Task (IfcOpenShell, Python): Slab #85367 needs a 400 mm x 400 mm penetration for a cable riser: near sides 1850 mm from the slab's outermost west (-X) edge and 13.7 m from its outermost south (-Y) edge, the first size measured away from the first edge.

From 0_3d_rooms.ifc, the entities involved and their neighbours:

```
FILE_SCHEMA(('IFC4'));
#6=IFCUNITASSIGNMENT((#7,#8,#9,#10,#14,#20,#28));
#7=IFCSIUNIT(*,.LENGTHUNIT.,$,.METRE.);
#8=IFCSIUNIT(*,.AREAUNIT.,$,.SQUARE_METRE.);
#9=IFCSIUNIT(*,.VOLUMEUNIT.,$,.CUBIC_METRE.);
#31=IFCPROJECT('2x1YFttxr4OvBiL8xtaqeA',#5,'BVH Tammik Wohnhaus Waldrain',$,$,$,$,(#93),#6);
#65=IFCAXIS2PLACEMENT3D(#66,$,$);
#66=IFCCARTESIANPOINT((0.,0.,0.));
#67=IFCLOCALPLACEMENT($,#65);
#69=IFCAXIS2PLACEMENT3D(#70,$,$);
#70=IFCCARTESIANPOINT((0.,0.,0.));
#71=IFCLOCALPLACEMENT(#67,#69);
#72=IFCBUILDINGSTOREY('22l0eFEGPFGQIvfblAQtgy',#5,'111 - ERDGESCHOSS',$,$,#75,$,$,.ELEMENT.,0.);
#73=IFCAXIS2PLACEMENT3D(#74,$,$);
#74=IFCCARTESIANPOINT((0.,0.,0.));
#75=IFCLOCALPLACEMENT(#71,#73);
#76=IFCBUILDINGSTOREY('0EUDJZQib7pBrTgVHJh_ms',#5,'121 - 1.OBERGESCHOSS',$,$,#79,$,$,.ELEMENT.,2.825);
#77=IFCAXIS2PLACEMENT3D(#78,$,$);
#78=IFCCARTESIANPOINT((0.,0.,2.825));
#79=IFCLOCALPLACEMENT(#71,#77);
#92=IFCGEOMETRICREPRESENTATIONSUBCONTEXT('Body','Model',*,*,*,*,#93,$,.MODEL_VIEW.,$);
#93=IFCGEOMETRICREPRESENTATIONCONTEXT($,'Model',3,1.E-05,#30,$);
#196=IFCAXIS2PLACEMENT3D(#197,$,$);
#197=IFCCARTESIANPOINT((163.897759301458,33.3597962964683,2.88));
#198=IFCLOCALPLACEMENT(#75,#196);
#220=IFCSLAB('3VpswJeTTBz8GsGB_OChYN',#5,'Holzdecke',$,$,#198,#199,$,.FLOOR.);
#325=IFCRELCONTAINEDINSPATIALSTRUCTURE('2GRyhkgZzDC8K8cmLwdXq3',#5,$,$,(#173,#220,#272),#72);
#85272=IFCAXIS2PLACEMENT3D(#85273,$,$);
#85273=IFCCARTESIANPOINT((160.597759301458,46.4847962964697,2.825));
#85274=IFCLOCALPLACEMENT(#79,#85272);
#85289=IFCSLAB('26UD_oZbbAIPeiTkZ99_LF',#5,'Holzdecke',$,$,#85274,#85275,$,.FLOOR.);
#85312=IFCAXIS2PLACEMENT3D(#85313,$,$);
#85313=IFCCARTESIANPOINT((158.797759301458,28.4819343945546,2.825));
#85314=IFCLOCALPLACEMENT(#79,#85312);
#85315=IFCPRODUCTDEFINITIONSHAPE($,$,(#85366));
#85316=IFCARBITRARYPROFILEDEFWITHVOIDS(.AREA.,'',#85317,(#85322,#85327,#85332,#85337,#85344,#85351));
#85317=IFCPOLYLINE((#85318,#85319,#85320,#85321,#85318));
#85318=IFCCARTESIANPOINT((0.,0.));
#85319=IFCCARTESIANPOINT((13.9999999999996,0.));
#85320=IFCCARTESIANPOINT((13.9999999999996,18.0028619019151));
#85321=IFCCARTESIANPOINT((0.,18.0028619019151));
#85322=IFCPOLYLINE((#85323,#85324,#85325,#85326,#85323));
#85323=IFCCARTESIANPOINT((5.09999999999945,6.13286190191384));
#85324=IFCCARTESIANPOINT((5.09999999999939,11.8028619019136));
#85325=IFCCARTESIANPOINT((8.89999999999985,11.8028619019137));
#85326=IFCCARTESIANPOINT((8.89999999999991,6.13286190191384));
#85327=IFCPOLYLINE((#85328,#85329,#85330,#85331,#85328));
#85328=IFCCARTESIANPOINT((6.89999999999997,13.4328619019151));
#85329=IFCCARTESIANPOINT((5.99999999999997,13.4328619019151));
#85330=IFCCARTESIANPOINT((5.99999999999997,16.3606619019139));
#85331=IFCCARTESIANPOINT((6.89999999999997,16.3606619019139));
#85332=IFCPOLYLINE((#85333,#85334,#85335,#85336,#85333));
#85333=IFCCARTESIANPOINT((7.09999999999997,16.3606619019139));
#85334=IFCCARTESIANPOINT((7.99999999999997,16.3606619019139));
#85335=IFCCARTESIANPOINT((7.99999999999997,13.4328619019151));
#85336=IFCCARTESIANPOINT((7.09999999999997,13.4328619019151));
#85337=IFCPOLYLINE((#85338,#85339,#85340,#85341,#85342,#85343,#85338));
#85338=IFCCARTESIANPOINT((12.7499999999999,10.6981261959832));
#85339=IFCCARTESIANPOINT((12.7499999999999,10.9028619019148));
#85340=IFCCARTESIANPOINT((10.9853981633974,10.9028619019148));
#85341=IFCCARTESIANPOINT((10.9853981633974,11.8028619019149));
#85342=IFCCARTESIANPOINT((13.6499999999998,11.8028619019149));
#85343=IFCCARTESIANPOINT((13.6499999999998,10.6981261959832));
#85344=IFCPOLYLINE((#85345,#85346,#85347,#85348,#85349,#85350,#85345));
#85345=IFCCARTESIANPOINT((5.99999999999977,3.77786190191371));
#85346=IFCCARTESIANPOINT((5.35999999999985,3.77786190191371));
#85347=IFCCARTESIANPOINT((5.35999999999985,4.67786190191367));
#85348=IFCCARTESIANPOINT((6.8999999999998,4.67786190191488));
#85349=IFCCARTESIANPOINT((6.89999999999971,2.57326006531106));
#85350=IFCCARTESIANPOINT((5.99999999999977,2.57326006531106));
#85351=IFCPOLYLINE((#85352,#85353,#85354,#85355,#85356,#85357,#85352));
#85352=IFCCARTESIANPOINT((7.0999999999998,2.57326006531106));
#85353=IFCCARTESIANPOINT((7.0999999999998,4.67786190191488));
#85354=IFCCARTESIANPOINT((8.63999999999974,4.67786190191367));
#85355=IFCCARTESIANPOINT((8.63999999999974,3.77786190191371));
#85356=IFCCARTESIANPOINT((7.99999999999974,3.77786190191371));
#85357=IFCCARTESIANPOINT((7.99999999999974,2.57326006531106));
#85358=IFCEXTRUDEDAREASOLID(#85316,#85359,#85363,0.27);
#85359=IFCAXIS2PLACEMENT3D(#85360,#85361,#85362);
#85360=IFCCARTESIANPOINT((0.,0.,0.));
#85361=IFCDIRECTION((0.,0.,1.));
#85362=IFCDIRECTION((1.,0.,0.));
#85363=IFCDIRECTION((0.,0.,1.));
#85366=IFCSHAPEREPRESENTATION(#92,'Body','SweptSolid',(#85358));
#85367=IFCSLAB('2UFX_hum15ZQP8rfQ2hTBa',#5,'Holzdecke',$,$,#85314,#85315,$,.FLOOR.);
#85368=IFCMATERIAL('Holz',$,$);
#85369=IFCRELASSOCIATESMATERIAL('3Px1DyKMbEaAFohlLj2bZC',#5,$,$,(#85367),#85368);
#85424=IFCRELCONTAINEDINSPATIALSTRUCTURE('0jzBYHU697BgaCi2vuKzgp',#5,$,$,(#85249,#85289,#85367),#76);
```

```python
import numpy as np
import ifcopenshell
import ifcopenshell.api.feature
import ifcopenshell.api.geometry
import ifcopenshell.api.root
import ifcopenshell.geom
import ifcopenshell.util.placement
import ifcopenshell.util.representation
import ifcopenshell.util.shape
import ifcopenshell.util.unit

model = ifcopenshell.open("0_3d_rooms.ifc")
unit_scale = ifcopenshell.util.unit.calculate_unit_scale(model)
settings = ifcopenshell.geom.settings()


def volume(element):
    """Net volume in cubic metres, openings subtracted."""
    shape = ifcopenshell.geom.create_shape(settings, element)
    return ifcopenshell.util.shape.get_volume(shape.geometry)


slab = model.by_id(85367)
before = volume(slab)

# Extent in the slab's own axes, in metres. The edges named are its -X and -Y sides.
slab_shape = ifcopenshell.geom.create_shape(settings, slab)
vertices = ifcopenshell.util.shape.get_vertices(slab_shape.geometry)
x_min, y_min, bottom = vertices.min(axis=0)
top = vertices[:, 2].max()

opening = ifcopenshell.api.root.create_entity(model, ifc_class="IfcOpeningElement", name="Cable riser opening", predefined_type="OPENING")
context = ifcopenshell.util.representation.get_context(model, "Model", "Body", "MODEL_VIEW")
width, depth = 0.4, 0.4
outline = [(0.0, 0.0), (width, 0.0), (width, depth), (0.0, depth), (0.0, 0.0)]
# Overshoot both faces by 50 mm so the cut is clean.
shape = ifcopenshell.api.geometry.add_slab_representation(
    model, context=context, depth=top - bottom + 0.1, polyline=outline
)
ifcopenshell.api.geometry.assign_representation(model, product=opening, representation=shape)

matrix = ifcopenshell.util.placement.get_local_placement(slab.ObjectPlacement)
matrix[:, 3] = matrix @ np.append(np.array([x_min + 1.85, y_min + 13.7, bottom - 0.05]) / unit_scale, 1.0)
ifcopenshell.api.geometry.edit_object_placement(model, product=opening, matrix=matrix, is_si=False)
ifcopenshell.api.feature.add_feature(model, feature=opening, element=slab)

after = volume(slab)

print(f"slab volume {before:.3f} -> {after:.3f} m3")

model.write("0_3d_rooms_v2.ifc")
```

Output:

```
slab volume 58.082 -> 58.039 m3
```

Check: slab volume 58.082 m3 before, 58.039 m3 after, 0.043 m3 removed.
